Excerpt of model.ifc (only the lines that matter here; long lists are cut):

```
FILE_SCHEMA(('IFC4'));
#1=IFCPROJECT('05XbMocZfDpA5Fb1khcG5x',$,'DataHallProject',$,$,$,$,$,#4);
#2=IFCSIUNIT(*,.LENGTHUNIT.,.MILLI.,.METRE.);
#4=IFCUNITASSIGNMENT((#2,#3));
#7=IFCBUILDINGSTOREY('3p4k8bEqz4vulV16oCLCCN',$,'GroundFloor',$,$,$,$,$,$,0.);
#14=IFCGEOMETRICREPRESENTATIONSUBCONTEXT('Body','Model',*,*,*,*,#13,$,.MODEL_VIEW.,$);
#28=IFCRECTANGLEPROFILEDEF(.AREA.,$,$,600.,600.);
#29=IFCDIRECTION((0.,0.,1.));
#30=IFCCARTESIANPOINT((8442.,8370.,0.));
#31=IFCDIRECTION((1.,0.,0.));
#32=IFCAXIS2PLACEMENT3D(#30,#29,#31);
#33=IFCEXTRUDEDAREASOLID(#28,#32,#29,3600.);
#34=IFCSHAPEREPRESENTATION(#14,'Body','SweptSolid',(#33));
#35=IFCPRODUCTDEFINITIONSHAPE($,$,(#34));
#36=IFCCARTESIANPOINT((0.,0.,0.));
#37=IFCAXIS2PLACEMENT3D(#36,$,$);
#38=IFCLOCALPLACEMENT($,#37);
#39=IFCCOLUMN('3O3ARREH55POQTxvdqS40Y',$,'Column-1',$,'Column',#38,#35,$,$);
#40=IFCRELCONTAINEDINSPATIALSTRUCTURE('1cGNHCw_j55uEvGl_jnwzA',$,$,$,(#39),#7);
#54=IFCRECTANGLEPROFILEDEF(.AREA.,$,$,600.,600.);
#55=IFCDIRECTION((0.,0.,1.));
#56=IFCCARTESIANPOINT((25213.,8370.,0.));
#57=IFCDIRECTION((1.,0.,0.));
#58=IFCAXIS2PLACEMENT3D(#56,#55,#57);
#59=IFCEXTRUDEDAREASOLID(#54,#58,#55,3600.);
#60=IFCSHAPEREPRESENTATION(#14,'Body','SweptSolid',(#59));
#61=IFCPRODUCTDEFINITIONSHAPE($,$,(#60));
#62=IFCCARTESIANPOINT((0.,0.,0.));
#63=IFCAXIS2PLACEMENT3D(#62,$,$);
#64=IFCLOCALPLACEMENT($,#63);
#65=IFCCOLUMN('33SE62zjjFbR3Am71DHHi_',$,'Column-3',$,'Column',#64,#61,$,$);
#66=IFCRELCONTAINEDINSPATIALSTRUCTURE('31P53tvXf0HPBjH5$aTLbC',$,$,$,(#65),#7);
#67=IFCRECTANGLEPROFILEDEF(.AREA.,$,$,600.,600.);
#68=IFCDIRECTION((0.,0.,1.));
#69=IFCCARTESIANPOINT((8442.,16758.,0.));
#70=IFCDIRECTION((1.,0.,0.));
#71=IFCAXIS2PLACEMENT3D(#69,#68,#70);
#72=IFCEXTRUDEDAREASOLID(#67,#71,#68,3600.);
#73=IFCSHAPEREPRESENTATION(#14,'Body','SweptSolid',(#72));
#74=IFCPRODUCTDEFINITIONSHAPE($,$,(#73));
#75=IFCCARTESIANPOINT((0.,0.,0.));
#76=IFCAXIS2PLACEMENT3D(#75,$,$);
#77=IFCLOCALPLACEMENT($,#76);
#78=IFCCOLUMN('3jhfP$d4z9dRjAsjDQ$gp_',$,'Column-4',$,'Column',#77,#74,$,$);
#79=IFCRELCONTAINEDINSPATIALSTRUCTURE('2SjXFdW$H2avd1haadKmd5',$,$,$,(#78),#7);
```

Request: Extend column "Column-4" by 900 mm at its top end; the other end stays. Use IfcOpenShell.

```python
import ifcopenshell
import ifcopenshell.util.representation
import ifcopenshell.util.unit

model = ifcopenshell.open("model.ifc")
unit_scale = ifcopenshell.util.unit.calculate_unit_scale(model)

member = model.by_guid("3jhfP$d4z9dRjAsjDQ$gp_")
change = 0.9 / unit_scale

# The extrusion runs towards the end named, so only its depth changes.
body = ifcopenshell.util.representation.get_representation(member, "Model", "Body")
solid = body.Items[0]
old_length = solid.Depth
solid.Depth += change

print(f"length {old_length:g} -> {solid.Depth:g}")

model.write("model-out.ifc")
```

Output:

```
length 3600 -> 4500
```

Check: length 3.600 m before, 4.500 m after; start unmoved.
